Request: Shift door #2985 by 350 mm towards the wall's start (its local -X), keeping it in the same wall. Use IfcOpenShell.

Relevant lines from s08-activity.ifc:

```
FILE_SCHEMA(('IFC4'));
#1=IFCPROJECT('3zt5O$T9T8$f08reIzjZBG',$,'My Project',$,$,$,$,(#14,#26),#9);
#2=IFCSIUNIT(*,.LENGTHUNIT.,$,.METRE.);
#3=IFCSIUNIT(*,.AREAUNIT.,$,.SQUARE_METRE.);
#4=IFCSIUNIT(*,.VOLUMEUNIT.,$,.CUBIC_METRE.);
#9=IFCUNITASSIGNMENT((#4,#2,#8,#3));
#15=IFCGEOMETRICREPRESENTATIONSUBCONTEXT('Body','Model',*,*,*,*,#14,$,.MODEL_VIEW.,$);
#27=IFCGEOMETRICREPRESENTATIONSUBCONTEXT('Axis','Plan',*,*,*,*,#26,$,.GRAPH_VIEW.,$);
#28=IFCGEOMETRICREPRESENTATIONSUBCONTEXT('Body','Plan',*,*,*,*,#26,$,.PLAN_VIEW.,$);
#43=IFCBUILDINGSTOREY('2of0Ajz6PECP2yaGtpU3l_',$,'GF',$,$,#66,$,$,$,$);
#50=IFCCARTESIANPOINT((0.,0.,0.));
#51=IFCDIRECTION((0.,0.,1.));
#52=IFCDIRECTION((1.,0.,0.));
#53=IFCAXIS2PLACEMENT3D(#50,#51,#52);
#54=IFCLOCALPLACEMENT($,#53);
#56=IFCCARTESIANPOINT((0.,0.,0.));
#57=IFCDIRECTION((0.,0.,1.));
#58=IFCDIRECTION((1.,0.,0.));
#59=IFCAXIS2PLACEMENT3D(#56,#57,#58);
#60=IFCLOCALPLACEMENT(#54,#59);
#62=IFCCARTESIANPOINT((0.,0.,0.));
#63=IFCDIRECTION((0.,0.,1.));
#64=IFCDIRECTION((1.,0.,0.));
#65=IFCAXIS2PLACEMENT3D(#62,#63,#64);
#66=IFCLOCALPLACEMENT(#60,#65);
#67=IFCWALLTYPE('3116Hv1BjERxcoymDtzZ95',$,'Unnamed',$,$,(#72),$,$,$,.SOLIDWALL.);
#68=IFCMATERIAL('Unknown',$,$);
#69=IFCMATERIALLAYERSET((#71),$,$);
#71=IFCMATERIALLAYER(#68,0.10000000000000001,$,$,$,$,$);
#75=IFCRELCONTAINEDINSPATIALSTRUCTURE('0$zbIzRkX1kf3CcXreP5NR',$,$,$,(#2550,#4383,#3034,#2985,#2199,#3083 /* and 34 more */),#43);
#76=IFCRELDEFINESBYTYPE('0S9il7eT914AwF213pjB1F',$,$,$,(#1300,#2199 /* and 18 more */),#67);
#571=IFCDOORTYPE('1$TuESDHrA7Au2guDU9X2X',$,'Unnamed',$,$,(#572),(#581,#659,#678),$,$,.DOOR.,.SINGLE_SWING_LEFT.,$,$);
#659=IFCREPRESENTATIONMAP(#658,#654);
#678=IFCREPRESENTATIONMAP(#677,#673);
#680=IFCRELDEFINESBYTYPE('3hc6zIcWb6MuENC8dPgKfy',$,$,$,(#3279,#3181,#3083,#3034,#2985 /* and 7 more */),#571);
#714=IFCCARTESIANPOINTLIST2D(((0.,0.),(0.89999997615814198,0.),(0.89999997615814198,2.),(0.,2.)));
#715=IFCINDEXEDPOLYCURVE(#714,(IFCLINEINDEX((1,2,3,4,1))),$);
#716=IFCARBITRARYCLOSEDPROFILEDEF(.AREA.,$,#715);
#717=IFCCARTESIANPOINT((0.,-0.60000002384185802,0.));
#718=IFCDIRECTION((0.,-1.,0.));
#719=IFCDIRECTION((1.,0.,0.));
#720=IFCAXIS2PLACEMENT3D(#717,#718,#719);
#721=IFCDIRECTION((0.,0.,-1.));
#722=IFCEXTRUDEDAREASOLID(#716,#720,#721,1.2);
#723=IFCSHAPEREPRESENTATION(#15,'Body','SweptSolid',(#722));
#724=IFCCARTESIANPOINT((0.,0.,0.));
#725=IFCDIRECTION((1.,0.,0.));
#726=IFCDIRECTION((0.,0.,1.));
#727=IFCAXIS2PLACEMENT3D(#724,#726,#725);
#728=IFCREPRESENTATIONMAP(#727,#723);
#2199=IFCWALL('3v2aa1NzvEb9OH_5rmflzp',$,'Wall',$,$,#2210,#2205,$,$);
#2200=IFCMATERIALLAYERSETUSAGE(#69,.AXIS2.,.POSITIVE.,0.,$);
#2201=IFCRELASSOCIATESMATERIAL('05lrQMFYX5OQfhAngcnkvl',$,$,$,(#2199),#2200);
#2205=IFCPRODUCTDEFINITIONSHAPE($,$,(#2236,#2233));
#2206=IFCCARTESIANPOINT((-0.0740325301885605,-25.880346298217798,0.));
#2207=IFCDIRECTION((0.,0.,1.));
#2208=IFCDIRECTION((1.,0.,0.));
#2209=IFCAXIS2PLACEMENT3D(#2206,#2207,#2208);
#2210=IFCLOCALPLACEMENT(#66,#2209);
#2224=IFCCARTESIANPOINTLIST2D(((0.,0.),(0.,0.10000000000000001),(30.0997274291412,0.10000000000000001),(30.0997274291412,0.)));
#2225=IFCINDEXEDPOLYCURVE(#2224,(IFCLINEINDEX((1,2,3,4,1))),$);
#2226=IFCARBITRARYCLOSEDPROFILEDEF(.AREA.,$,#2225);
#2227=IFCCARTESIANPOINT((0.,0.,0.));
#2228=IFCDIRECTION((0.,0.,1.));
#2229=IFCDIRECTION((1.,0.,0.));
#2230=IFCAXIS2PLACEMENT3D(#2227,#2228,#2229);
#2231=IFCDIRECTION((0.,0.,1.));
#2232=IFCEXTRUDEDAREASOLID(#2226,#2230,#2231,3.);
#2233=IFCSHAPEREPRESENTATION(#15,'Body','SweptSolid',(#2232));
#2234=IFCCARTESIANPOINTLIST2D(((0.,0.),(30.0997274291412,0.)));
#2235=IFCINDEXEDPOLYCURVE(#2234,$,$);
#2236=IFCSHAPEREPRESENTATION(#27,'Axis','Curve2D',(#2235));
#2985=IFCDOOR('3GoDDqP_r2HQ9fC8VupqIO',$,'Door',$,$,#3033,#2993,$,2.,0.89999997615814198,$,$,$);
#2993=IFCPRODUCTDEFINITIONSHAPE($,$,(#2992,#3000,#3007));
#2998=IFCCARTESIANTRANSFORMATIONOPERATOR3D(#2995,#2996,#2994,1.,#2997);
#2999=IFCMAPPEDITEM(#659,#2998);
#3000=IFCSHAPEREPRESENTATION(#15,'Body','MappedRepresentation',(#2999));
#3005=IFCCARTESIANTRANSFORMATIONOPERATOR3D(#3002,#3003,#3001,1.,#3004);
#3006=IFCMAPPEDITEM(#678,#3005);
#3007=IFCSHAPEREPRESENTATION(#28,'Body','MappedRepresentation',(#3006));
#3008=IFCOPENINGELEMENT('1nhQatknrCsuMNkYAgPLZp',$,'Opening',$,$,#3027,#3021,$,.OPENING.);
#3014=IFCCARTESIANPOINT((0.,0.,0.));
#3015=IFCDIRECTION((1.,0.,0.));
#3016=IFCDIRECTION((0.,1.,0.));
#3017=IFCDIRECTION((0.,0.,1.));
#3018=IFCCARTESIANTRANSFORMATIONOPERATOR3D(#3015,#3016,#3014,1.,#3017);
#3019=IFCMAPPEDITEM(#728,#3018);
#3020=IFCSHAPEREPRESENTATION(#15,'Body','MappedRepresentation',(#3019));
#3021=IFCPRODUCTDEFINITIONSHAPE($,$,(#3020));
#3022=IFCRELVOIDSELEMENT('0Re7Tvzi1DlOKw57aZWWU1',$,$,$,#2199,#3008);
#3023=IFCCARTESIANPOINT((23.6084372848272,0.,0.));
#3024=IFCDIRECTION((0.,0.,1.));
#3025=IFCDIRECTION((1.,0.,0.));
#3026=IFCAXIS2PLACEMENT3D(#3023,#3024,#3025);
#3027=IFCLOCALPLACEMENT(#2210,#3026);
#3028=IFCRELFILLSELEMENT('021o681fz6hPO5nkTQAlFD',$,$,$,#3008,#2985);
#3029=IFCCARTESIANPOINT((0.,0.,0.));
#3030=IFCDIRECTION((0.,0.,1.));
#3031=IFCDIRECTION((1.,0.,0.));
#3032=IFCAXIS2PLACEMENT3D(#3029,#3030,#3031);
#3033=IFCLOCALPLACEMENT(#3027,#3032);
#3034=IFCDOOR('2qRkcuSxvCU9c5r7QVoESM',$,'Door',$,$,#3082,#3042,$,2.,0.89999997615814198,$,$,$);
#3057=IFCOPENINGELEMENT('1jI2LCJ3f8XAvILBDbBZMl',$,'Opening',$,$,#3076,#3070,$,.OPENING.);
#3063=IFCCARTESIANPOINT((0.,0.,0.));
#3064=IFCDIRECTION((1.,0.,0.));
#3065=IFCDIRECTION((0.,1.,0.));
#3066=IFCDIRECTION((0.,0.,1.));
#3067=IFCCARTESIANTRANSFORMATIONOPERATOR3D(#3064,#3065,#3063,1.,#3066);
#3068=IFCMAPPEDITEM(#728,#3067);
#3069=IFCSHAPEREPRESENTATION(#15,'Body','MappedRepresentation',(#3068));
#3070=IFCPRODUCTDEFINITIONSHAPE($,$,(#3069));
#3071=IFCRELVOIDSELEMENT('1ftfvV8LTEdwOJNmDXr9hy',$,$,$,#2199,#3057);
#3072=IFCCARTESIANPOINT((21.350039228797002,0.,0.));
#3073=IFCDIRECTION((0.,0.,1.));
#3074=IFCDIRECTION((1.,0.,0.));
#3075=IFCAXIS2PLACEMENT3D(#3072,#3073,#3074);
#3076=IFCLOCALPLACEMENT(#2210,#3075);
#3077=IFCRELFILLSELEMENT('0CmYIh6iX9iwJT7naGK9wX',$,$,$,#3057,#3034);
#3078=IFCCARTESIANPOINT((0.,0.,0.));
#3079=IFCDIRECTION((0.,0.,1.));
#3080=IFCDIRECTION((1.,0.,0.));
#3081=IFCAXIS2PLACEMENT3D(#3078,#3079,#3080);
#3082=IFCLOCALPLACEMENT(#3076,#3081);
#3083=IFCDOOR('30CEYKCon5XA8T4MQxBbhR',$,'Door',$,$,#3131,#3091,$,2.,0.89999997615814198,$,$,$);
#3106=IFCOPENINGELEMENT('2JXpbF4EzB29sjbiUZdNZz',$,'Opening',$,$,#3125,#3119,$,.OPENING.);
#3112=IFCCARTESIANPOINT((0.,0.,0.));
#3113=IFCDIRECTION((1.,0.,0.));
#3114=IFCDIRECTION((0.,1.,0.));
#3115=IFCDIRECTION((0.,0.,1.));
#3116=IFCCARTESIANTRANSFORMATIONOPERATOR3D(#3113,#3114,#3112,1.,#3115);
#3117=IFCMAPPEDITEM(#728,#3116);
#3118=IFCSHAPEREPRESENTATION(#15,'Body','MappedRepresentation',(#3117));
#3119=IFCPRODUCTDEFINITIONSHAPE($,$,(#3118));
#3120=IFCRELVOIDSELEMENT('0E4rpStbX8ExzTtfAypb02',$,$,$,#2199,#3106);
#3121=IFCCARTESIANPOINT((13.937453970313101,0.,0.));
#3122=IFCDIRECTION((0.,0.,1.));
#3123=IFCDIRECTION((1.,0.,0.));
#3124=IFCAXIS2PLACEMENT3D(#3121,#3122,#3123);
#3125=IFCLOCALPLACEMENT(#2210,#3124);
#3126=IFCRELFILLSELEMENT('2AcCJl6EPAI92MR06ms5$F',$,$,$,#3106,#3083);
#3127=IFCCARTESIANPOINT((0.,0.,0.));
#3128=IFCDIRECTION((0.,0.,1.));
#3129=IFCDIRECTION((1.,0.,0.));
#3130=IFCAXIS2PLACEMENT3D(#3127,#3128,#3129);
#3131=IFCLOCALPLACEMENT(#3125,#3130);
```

```python
import ifcopenshell
import ifcopenshell.api.geometry
import ifcopenshell.util.placement
import ifcopenshell.util.unit

model = ifcopenshell.open("s08-activity.ifc")
unit_scale = ifcopenshell.util.unit.calculate_unit_scale(model)

door = model.by_id(2985)
opening = door.FillsVoids[0].RelatingOpeningElement
wall = opening.VoidsElements[0].RelatingBuildingElement

wall_matrix = ifcopenshell.util.placement.get_local_placement(wall.ObjectPlacement)
shift = wall_matrix[:3, 0] * -0.35 / unit_scale
before = ifcopenshell.util.placement.get_local_placement(door.ObjectPlacement)[:3, 3].copy()

# The door is placed relative to its opening, so it follows when the opening moves.
matrix = ifcopenshell.util.placement.get_local_placement(opening.ObjectPlacement)
matrix[:3, 3] += shift
ifcopenshell.api.geometry.edit_object_placement(
    model, product=opening, matrix=matrix, is_si=False, should_transform_children=True
)

after = ifcopenshell.util.placement.get_local_placement(door.ObjectPlacement)[:3, 3]
print("door moved by", (after - before).round(3) + 0.0)

model.write("s08-activity_rev.ifc")
```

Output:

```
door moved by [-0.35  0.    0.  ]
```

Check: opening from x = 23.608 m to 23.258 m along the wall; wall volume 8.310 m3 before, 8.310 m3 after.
